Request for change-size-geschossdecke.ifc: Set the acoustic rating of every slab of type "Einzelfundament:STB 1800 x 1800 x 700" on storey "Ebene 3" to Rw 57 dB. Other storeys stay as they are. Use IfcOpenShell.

First a look at what the model holds.

```python
import ifcopenshell
import ifcopenshell.util.element

model = ifcopenshell.open("change-size-geschossdecke.ifc")
print(model.schema)
storey = next(s for s in model.by_type("IfcBuildingStorey") if s.Name == "Ebene 3")
slabs = [e for e in ifcopenshell.util.element.get_decomposition(storey) if e.is_a("IfcSlab")]
seen = {}
for e in slabs:
    element_type = ifcopenshell.util.element.get_type(e)
    key = (element_type.Name if element_type != e and element_type else None, ifcopenshell.util.element.get_pset(e, "Pset_SlabCommon", "AcousticRating"))
    seen[key] = seen.get(key, 0) + 1
for (name, value), count in sorted(seen.items(), key=str):
    print(count, "x", name, "|", value)
```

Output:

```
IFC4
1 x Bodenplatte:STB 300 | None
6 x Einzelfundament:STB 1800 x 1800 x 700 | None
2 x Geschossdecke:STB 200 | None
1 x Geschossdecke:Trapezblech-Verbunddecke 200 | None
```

```python
import ifcopenshell
import ifcopenshell.api.pset
import ifcopenshell.util.element

model = ifcopenshell.open("change-size-geschossdecke.ifc")

storey = next(s for s in model.by_type("IfcBuildingStorey") if s.Name == "Ebene 3")
slabs = [e for e in ifcopenshell.util.element.get_decomposition(storey) if e.is_a("IfcSlab")]

count = 0
for e in slabs:
    element_type = ifcopenshell.util.element.get_type(e)
    if element_type in (None, e) or element_type.Name != "Einzelfundament:STB 1800 x 1800 x 700":
        continue
    # add_pset returns the element's existing set when there is one.
    pset = ifcopenshell.api.pset.add_pset(model, product=e, name="Pset_SlabCommon")
    ifcopenshell.api.pset.edit_pset(model, pset=pset, properties={"AcousticRating": "Rw 57 dB"})
    count += 1

print(count, "slabs updated")

model.write("change-size-geschossdecke_rev.ifc")
```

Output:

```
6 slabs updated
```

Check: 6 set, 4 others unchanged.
